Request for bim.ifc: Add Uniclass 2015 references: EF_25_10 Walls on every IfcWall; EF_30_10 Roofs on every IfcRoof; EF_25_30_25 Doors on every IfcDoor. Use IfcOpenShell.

First a look at what the model holds.

```python
import ifcopenshell

model = ifcopenshell.open("bim.ifc")
print(model.schema)
print("classifications:", [c.Name for c in model.by_type("IfcClassification")])
for ifc_class in ("IfcDoor", "IfcRoof", "IfcStair", "IfcWall", "IfcWindow"):
    print(ifc_class, len(model.by_type(ifc_class)))
```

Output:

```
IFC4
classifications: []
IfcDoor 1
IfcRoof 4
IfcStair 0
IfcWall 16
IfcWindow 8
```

```python
import ifcopenshell
import ifcopenshell.api.classification

model = ifcopenshell.open("bim.ifc")

system = ifcopenshell.api.classification.add_classification(model, classification="Uniclass 2015")

codes = {
    "IfcWall": ("EF_25_10", "Walls"),
    "IfcRoof": ("EF_30_10", "Roofs"),
    "IfcDoor": ("EF_25_30_25", "Doors"),
}
for ifc_class, (code, name) in codes.items():
    products = model.by_type(ifc_class)
    ifcopenshell.api.classification.add_reference(
        model, products=products, classification=system, identification=code, name=name
    )
    print(code, len(products))

model.write("bim_updated.ifc")
```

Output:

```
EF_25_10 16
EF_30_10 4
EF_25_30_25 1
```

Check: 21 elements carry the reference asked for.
